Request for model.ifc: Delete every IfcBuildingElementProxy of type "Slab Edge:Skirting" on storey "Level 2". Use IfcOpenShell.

First a look at what the model holds.

```python
import ifcopenshell
import ifcopenshell.util.element

model = ifcopenshell.open("model.ifc")
print(model.schema)
storey = next(s for s in model.by_type("IfcBuildingStorey") if s.Name == "Level 2")
proxies = [e for e in ifcopenshell.util.element.get_decomposition(storey) if e.is_a("IfcBuildingElementProxy")]
seen = {}
for e in proxies:
    element_type = ifcopenshell.util.element.get_type(e)
    name = element_type.Name if element_type not in (None, e) else None
    seen[name] = seen.get(name, 0) + 1
for name, count in sorted(seen.items(), key=str):
    print(count, "x", name)
```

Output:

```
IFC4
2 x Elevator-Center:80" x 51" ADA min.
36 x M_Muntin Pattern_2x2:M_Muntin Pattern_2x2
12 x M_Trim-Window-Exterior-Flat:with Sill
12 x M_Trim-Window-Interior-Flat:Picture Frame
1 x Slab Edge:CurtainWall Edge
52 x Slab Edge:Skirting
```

```python
import ifcopenshell
import ifcopenshell.api.root
import ifcopenshell.util.element

model = ifcopenshell.open("model.ifc")

storey = next(s for s in model.by_type("IfcBuildingStorey") if s.Name == "Level 2")
proxies = [e for e in ifcopenshell.util.element.get_decomposition(storey) if e.is_a("IfcBuildingElementProxy")]
targets = [e for e in proxies if (t := ifcopenshell.util.element.get_type(e)) not in (None, e) and t.Name == "Slab Edge:Skirting"]

for e in targets:
    ifcopenshell.api.root.remove_product(model, product=e)
print(len(targets), "removed")

model.write("model_rev.ifc")
```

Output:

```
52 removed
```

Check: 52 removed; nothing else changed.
